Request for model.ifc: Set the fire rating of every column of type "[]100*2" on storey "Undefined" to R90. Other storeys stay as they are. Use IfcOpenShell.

First a look at what the model holds.

```python
import ifcopenshell
import ifcopenshell.util.element

model = ifcopenshell.open("model.ifc")
print(model.schema)
storey = next(s for s in model.by_type("IfcBuildingStorey") if s.Name == "Undefined")
columns = [e for e in ifcopenshell.util.element.get_decomposition(storey) if e.is_a("IfcColumn")]
seen = {}
for e in columns:
    element_type = ifcopenshell.util.element.get_type(e)
    key = (element_type.Name if element_type != e and element_type else None, ifcopenshell.util.element.get_pset(e, "Pset_ColumnCommon", "FireRating"))
    seen[key] = seen.get(key, 0) + 1
for (name, value), count in sorted(seen.items(), key=str):
    print(count, "x", name, "|", value)
```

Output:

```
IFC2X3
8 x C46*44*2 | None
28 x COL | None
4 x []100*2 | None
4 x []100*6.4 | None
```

```python
import ifcopenshell
import ifcopenshell.api.pset
import ifcopenshell.util.element

model = ifcopenshell.open("model.ifc")

storey = next(s for s in model.by_type("IfcBuildingStorey") if s.Name == "Undefined")
columns = [e for e in ifcopenshell.util.element.get_decomposition(storey) if e.is_a("IfcColumn")]

count = 0
for e in columns:
    element_type = ifcopenshell.util.element.get_type(e)
    if element_type in (None, e) or element_type.Name != "[]100*2":
        continue
    found = ifcopenshell.util.element.get_pset(e, "Pset_ColumnCommon", should_inherit=False)
    if found:
        pset = model.by_id(found["id"])
        if len(ifcopenshell.util.element.get_elements_by_pset(pset)) > 1:
            pset = ifcopenshell.api.pset.unshare_pset(model, products=[e], pset=pset)[0]
    else:
        pset = ifcopenshell.api.pset.add_pset(model, product=e, name="Pset_ColumnCommon")
    ifcopenshell.api.pset.edit_pset(model, pset=pset, properties={"FireRating": "R90"})
    count += 1

print(count, "columns updated")

model.write("model_updated.ifc")
```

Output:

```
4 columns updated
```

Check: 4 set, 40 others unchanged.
